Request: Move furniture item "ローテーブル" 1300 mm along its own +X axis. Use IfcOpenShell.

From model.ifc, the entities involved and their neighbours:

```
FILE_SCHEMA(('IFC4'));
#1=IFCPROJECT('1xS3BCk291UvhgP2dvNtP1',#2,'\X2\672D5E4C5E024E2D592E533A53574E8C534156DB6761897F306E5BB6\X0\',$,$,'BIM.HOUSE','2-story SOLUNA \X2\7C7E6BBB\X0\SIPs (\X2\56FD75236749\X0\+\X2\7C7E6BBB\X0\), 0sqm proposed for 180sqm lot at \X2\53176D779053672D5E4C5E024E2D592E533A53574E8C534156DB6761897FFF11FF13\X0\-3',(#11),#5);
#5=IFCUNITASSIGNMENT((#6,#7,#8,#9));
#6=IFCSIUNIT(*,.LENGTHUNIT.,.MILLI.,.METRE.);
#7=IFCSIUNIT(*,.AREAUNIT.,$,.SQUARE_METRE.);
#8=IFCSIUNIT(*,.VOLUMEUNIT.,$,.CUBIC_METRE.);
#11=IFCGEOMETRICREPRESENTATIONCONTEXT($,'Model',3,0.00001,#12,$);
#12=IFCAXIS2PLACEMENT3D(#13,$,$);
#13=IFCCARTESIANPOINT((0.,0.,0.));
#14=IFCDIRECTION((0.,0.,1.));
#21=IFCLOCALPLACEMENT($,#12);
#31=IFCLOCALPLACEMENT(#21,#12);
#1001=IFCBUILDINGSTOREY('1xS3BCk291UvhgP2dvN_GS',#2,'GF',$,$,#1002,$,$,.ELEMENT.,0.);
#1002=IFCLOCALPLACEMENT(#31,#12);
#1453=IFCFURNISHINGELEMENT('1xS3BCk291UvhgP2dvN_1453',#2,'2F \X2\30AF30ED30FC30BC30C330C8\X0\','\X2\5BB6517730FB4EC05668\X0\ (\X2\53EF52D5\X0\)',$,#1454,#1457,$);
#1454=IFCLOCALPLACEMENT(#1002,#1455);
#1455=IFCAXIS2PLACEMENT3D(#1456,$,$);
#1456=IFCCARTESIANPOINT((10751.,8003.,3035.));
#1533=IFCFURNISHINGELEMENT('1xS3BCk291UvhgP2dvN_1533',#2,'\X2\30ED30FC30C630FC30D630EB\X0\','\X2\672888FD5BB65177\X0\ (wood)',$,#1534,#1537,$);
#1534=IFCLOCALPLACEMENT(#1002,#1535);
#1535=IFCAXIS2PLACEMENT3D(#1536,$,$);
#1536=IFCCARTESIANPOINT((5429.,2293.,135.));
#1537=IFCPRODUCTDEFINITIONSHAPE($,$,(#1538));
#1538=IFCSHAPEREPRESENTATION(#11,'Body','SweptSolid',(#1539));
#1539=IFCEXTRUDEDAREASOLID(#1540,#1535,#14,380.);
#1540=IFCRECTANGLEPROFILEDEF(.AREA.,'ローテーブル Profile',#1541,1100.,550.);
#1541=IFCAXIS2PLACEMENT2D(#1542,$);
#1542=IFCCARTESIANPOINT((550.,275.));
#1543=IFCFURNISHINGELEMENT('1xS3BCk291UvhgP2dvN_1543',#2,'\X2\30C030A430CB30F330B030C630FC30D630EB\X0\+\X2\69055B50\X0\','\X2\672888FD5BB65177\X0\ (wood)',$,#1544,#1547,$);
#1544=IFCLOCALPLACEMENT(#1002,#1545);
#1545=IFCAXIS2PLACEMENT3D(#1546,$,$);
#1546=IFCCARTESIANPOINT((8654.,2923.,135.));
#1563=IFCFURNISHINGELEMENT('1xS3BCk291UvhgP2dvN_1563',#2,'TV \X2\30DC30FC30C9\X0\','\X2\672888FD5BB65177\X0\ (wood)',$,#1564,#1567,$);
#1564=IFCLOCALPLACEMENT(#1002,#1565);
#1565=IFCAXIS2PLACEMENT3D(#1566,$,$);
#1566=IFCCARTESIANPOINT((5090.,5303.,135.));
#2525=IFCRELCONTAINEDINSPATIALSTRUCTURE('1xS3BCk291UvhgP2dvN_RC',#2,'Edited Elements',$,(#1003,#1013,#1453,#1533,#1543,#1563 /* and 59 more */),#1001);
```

```python
import ifcopenshell
import ifcopenshell.api.geometry
import ifcopenshell.util.placement
import ifcopenshell.util.unit

model = ifcopenshell.open("model.ifc")
unit_scale = ifcopenshell.util.unit.calculate_unit_scale(model)

item = model.by_guid("1xS3BCk291UvhgP2dvN_1533")
matrix = ifcopenshell.util.placement.get_local_placement(item.ObjectPlacement)
matrix[:3, 3] += matrix[:3, 0] * 1.3 / unit_scale
ifcopenshell.api.geometry.edit_object_placement(model, product=item, matrix=matrix, is_si=False)

print(ifcopenshell.util.placement.get_local_placement(item.ObjectPlacement).round(3) + 0.0)

model.write("model_edited.ifc")
```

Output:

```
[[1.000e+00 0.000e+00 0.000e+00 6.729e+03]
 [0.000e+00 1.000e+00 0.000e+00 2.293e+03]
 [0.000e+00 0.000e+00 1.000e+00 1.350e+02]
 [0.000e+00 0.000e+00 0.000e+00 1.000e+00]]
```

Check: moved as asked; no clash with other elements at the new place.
